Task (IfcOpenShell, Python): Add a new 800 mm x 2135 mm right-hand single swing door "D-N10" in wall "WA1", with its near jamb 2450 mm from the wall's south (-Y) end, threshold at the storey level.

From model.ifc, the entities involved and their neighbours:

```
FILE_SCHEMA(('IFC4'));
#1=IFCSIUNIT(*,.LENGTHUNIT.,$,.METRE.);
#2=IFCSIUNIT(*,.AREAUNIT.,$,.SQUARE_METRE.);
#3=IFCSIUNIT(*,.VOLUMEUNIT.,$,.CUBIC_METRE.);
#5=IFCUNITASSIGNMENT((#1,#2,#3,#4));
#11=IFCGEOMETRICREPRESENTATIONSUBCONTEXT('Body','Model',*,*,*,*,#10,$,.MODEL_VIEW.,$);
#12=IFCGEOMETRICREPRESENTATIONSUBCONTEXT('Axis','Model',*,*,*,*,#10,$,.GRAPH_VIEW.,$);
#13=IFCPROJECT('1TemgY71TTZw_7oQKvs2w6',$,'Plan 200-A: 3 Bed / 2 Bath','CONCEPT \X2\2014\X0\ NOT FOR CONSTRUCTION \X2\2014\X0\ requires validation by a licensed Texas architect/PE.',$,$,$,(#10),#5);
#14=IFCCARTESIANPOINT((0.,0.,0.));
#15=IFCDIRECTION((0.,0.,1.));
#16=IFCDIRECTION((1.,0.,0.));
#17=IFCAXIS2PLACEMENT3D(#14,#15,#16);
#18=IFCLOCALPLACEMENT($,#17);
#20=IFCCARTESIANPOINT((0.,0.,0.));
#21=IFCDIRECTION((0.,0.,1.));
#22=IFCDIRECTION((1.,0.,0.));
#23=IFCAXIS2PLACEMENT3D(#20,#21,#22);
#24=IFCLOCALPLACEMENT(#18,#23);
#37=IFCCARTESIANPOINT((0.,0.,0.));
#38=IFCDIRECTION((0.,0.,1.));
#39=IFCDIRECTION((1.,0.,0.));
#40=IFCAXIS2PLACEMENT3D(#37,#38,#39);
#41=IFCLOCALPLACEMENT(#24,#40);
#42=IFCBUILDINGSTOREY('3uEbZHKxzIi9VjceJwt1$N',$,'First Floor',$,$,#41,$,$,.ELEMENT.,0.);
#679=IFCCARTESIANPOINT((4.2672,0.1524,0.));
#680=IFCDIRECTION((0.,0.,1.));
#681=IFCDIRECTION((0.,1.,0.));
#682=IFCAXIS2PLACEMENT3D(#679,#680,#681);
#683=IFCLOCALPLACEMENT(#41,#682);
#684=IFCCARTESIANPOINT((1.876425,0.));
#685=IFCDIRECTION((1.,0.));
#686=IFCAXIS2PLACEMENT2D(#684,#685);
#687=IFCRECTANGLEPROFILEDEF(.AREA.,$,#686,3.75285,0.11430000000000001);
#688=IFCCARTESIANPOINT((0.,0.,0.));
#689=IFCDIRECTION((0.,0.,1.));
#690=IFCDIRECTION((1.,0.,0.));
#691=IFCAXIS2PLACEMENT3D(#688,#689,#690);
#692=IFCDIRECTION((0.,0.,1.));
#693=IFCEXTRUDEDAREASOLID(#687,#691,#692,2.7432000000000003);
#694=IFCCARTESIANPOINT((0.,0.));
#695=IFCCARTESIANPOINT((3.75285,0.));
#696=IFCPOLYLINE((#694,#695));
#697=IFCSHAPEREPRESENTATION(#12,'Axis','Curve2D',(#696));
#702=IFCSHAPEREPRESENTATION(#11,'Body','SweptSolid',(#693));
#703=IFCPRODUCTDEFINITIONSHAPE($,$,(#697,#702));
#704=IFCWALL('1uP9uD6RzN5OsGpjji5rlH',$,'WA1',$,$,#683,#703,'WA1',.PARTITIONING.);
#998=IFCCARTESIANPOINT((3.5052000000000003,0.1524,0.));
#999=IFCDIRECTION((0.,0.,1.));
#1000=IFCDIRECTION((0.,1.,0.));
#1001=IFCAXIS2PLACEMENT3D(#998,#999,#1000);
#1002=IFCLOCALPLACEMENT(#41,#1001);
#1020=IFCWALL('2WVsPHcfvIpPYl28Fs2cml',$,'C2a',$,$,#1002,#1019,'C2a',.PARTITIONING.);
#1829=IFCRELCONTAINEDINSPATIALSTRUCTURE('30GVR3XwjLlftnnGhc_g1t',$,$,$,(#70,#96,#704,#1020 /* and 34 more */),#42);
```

```python
import numpy as np
import ifcopenshell
import ifcopenshell.api.feature
import ifcopenshell.api.geometry
import ifcopenshell.api.root
import ifcopenshell.api.spatial
import ifcopenshell.geom
import ifcopenshell.util.element
import ifcopenshell.util.placement
import ifcopenshell.util.representation
import ifcopenshell.util.shape
import ifcopenshell.util.unit

model = ifcopenshell.open("model.ifc")
unit_scale = ifcopenshell.util.unit.calculate_unit_scale(model)
settings = ifcopenshell.geom.settings()


def volume(element):
    """Net volume in cubic metres, openings subtracted."""
    shape = ifcopenshell.geom.create_shape(settings, element)
    return ifcopenshell.util.shape.get_volume(shape.geometry)


wall = model.by_id(704)
storey = ifcopenshell.util.element.get_container(wall, ifc_class="IfcBuildingStorey")
context = ifcopenshell.util.representation.get_context(model, "Model", "Body", "MODEL_VIEW")
before = volume(wall)

width, height, from_end, sill = 0.8, 2.135, 2.45, 0.0  # metres

# The wall runs along its own X axis, and the end named is its -X end.
wall_shape = ifcopenshell.geom.create_shape(settings, wall)
x, y, z = ifcopenshell.util.shape.get_vertices(wall_shape.geometry).T
start = x.min() + from_end
face, thickness = float(y.min()), float(y.max() - y.min())
wall_matrix = ifcopenshell.util.placement.get_local_placement(wall.ObjectPlacement)
level = ifcopenshell.util.placement.get_local_placement(storey.ObjectPlacement)[2, 3]


def in_wall(x, y):
    """Placement at x, y metres in the wall's axes, at sill height."""
    matrix = wall_matrix.copy()
    matrix[:, 3] = wall_matrix @ np.array([x / unit_scale, y / unit_scale, 0.0, 1.0])
    matrix[2, 3] = level + sill / unit_scale
    return matrix


# Opening: a box that overshoots both wall faces by 50 mm.
opening = ifcopenshell.api.root.create_entity(model, ifc_class="IfcOpeningElement", predefined_type="OPENING")
box = ifcopenshell.api.geometry.add_wall_representation(
    model, context=context, length=width, height=height, thickness=thickness + 0.1
)
ifcopenshell.api.geometry.assign_representation(model, product=opening, representation=box)
ifcopenshell.api.geometry.edit_object_placement(model, product=opening, matrix=in_wall(start, face - 0.05), is_si=False)
ifcopenshell.api.feature.add_feature(model, feature=opening, element=wall)

door = ifcopenshell.api.root.create_entity(model, ifc_class="IfcDoor", name="D-N10", predefined_type="DOOR")
door.OverallWidth, door.OverallHeight = width / unit_scale, height / unit_scale
door.OperationType = "SINGLE_SWING_RIGHT"
body = ifcopenshell.api.geometry.add_door_representation(
    model,
    context=context,
    overall_width=door.OverallWidth,
    overall_height=door.OverallHeight,
    operation_type="SINGLE_SWING_RIGHT",
    lining_properties={"LiningDepth": thickness / unit_scale, "ThresholdDepth": thickness / unit_scale},
)
ifcopenshell.api.geometry.assign_representation(model, product=door, representation=body)
ifcopenshell.api.spatial.assign_container(model, products=[door], relating_structure=storey)
ifcopenshell.api.feature.add_filling(model, opening=opening, element=door)

# The lining spans the wall, so the door starts at the wall face.
ifcopenshell.api.geometry.edit_object_placement(model, product=door, matrix=in_wall(start, face), is_si=False)

after = volume(wall)

print(f"wall volume {before:.3f} -> {after:.3f} m3")

model.write("model_rev.ifc")
```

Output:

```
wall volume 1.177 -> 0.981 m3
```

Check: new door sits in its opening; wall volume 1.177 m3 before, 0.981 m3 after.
